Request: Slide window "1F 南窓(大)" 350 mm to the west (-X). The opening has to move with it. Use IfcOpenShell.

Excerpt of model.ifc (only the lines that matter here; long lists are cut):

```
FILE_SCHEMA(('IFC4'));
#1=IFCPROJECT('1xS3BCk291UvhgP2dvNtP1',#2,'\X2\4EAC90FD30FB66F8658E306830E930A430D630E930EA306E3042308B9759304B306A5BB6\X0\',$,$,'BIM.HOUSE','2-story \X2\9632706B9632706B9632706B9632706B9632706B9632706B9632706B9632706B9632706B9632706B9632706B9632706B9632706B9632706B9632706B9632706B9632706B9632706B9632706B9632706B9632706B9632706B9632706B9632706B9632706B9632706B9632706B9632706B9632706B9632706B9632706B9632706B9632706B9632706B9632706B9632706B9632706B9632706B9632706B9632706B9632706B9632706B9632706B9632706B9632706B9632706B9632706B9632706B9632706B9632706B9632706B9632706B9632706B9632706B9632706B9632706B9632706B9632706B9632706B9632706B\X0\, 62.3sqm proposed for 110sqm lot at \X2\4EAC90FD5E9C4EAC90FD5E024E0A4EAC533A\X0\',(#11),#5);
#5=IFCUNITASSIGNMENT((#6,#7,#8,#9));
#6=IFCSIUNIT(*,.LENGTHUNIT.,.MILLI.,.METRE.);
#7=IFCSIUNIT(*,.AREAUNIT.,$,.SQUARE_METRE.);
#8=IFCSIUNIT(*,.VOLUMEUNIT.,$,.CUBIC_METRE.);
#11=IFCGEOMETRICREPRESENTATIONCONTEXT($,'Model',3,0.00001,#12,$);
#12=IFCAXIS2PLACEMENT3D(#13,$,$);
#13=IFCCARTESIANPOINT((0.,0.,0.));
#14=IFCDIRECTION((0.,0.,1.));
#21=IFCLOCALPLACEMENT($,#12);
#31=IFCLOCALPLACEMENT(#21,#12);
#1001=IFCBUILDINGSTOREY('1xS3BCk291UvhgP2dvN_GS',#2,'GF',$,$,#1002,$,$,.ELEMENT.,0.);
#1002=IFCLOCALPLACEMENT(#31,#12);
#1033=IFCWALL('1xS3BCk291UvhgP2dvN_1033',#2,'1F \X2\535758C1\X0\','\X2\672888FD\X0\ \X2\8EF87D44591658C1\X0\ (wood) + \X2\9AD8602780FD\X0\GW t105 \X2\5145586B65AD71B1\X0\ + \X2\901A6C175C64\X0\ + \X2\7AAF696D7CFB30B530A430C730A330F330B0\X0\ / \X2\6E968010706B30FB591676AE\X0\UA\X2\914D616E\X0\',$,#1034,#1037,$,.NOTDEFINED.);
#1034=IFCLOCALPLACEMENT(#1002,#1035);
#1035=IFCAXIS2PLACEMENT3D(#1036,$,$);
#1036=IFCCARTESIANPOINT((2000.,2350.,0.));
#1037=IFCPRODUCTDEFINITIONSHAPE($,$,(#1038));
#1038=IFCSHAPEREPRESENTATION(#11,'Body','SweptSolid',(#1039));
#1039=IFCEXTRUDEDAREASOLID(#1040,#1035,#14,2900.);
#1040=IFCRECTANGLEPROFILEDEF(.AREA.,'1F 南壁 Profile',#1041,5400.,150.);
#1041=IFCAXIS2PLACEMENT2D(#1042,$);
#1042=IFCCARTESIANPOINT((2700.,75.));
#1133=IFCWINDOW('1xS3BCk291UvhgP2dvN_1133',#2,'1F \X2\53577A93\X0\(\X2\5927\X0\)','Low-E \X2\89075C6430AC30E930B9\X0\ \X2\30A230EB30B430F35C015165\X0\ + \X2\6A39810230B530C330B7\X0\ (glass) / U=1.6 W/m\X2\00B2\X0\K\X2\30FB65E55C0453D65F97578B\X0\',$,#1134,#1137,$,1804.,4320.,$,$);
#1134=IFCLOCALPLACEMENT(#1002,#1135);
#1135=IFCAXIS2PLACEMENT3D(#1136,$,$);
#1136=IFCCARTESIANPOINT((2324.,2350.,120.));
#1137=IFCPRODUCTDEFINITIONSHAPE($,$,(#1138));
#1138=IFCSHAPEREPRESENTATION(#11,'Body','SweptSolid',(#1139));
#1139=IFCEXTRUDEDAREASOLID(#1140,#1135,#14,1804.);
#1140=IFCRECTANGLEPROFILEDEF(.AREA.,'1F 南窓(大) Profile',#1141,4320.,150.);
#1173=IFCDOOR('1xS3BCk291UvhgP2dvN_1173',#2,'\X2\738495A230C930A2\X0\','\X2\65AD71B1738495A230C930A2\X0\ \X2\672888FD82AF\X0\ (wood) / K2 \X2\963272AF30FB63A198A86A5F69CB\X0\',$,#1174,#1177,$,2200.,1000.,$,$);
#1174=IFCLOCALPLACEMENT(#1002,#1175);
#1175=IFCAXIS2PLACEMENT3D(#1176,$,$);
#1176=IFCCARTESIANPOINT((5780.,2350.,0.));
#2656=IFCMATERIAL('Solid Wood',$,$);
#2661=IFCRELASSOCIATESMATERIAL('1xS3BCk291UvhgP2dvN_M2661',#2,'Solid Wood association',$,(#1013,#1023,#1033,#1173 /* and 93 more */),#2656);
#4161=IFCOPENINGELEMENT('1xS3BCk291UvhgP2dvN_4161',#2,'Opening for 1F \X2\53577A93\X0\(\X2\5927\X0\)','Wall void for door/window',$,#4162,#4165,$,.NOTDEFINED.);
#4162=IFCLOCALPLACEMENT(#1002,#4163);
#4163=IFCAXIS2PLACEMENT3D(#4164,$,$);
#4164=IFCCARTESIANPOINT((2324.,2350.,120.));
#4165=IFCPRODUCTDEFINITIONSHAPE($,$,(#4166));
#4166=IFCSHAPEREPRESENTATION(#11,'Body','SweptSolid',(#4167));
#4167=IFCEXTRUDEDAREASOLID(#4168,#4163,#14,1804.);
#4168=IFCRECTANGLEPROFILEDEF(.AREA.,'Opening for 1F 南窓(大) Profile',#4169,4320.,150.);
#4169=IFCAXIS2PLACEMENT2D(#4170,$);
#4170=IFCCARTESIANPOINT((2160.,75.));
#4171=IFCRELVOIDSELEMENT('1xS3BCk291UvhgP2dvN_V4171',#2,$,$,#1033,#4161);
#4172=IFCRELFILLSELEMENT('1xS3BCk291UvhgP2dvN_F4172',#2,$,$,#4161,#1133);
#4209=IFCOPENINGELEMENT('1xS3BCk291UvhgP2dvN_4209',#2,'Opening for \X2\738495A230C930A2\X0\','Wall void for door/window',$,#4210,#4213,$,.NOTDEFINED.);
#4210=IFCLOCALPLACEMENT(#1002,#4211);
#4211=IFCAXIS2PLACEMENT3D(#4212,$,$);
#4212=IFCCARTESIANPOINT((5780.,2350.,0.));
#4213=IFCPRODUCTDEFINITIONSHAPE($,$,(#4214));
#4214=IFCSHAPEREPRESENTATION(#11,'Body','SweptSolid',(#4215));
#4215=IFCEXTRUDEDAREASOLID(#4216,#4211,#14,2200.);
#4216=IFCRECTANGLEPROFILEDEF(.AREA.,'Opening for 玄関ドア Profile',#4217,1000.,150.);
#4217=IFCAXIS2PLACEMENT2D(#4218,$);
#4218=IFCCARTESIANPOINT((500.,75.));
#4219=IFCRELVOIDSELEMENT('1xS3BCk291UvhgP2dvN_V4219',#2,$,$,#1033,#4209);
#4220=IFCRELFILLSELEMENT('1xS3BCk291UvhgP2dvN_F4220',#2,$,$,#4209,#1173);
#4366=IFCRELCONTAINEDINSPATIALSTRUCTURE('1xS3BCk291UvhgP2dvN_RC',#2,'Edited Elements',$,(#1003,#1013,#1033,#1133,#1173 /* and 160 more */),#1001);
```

```python
import ifcopenshell
import ifcopenshell.api.geometry
import ifcopenshell.util.placement
import ifcopenshell.util.unit

model = ifcopenshell.open("model.ifc")
unit_scale = ifcopenshell.util.unit.calculate_unit_scale(model)

window = model.by_guid("1xS3BCk291UvhgP2dvN_1133")
opening = window.FillsVoids[0].RelatingOpeningElement
wall = opening.VoidsElements[0].RelatingBuildingElement

wall_matrix = ifcopenshell.util.placement.get_local_placement(wall.ObjectPlacement)
shift = wall_matrix[:3, 0] * -0.35 / unit_scale
before = ifcopenshell.util.placement.get_local_placement(window.ObjectPlacement)[:3, 3].copy()

# The window is not placed relative to its opening, so move both.
for product in (opening, window):
    matrix = ifcopenshell.util.placement.get_local_placement(product.ObjectPlacement)
    matrix[:3, 3] += shift
    ifcopenshell.api.geometry.edit_object_placement(model, product=product, matrix=matrix, is_si=False)

after = ifcopenshell.util.placement.get_local_placement(window.ObjectPlacement)[:3, 3]
print("window moved by", (after - before).round(3) + 0.0)

model.write("model-out.ifc")
```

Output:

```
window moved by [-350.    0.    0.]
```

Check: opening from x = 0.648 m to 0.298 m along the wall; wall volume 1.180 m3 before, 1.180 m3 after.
